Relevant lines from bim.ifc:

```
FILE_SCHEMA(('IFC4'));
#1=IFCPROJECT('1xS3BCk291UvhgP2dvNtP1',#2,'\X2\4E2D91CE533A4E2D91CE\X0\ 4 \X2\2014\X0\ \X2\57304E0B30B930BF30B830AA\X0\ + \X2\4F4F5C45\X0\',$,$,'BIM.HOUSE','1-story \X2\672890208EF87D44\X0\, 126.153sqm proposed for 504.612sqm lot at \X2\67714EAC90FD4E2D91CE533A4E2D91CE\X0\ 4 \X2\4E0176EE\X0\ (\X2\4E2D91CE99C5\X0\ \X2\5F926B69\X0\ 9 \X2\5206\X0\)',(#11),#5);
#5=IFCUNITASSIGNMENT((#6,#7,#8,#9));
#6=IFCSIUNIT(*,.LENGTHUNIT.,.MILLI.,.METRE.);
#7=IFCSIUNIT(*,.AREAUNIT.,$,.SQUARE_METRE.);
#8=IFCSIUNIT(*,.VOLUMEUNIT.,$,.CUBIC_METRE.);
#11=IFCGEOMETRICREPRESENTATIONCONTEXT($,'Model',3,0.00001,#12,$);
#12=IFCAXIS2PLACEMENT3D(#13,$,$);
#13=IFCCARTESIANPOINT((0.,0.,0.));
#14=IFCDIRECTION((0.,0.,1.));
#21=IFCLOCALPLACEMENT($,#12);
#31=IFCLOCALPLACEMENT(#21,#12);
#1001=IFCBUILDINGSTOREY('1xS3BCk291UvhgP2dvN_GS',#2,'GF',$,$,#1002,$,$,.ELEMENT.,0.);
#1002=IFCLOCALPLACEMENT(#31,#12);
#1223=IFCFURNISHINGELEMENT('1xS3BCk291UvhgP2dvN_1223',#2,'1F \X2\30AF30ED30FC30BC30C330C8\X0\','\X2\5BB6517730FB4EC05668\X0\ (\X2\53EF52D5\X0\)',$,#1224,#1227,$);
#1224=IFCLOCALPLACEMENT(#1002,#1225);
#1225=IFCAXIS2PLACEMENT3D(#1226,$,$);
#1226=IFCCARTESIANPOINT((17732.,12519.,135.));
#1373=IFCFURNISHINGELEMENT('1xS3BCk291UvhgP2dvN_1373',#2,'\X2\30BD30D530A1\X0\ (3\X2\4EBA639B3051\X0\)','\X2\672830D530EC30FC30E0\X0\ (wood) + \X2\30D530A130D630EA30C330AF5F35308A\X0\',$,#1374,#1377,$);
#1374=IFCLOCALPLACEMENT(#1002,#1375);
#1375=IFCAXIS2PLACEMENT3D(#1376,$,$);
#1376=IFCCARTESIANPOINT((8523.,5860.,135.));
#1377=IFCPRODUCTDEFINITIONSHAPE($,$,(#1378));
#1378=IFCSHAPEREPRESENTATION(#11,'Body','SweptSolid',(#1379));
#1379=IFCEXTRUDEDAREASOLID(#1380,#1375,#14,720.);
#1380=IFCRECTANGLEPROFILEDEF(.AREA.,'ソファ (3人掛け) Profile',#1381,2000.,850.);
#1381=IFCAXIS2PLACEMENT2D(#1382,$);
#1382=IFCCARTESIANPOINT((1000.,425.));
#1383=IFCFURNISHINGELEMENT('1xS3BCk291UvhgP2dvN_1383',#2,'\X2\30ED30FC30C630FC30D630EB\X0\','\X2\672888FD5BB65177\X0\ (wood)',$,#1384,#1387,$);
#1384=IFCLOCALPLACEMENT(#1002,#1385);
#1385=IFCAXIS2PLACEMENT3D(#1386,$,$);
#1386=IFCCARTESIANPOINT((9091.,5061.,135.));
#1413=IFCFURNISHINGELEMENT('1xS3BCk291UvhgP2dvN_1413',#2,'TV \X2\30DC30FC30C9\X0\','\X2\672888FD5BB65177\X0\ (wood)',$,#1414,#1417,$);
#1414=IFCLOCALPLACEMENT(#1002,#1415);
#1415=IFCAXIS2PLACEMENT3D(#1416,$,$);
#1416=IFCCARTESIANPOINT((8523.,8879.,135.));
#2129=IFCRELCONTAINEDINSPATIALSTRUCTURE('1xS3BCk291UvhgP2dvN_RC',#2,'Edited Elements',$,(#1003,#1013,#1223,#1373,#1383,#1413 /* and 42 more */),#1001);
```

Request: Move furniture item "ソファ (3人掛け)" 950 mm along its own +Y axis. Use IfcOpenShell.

```python
import ifcopenshell
import ifcopenshell.api.geometry
import ifcopenshell.util.placement

model = ifcopenshell.open("bim.ifc")

item = model.by_guid("1xS3BCk291UvhgP2dvN_1373")
matrix = ifcopenshell.util.placement.get_local_placement(item.ObjectPlacement)
matrix[:3, 3] += matrix[:3, 1] * 950.0
ifcopenshell.api.geometry.edit_object_placement(model, product=item, matrix=matrix, is_si=False)

print(ifcopenshell.util.placement.get_local_placement(item.ObjectPlacement).round(3) + 0.0)

model.write("bim_edited.ifc")
```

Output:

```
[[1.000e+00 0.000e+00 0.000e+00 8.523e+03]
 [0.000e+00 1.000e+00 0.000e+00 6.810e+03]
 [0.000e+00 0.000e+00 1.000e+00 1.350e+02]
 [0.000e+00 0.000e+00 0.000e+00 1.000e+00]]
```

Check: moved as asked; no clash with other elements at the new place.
